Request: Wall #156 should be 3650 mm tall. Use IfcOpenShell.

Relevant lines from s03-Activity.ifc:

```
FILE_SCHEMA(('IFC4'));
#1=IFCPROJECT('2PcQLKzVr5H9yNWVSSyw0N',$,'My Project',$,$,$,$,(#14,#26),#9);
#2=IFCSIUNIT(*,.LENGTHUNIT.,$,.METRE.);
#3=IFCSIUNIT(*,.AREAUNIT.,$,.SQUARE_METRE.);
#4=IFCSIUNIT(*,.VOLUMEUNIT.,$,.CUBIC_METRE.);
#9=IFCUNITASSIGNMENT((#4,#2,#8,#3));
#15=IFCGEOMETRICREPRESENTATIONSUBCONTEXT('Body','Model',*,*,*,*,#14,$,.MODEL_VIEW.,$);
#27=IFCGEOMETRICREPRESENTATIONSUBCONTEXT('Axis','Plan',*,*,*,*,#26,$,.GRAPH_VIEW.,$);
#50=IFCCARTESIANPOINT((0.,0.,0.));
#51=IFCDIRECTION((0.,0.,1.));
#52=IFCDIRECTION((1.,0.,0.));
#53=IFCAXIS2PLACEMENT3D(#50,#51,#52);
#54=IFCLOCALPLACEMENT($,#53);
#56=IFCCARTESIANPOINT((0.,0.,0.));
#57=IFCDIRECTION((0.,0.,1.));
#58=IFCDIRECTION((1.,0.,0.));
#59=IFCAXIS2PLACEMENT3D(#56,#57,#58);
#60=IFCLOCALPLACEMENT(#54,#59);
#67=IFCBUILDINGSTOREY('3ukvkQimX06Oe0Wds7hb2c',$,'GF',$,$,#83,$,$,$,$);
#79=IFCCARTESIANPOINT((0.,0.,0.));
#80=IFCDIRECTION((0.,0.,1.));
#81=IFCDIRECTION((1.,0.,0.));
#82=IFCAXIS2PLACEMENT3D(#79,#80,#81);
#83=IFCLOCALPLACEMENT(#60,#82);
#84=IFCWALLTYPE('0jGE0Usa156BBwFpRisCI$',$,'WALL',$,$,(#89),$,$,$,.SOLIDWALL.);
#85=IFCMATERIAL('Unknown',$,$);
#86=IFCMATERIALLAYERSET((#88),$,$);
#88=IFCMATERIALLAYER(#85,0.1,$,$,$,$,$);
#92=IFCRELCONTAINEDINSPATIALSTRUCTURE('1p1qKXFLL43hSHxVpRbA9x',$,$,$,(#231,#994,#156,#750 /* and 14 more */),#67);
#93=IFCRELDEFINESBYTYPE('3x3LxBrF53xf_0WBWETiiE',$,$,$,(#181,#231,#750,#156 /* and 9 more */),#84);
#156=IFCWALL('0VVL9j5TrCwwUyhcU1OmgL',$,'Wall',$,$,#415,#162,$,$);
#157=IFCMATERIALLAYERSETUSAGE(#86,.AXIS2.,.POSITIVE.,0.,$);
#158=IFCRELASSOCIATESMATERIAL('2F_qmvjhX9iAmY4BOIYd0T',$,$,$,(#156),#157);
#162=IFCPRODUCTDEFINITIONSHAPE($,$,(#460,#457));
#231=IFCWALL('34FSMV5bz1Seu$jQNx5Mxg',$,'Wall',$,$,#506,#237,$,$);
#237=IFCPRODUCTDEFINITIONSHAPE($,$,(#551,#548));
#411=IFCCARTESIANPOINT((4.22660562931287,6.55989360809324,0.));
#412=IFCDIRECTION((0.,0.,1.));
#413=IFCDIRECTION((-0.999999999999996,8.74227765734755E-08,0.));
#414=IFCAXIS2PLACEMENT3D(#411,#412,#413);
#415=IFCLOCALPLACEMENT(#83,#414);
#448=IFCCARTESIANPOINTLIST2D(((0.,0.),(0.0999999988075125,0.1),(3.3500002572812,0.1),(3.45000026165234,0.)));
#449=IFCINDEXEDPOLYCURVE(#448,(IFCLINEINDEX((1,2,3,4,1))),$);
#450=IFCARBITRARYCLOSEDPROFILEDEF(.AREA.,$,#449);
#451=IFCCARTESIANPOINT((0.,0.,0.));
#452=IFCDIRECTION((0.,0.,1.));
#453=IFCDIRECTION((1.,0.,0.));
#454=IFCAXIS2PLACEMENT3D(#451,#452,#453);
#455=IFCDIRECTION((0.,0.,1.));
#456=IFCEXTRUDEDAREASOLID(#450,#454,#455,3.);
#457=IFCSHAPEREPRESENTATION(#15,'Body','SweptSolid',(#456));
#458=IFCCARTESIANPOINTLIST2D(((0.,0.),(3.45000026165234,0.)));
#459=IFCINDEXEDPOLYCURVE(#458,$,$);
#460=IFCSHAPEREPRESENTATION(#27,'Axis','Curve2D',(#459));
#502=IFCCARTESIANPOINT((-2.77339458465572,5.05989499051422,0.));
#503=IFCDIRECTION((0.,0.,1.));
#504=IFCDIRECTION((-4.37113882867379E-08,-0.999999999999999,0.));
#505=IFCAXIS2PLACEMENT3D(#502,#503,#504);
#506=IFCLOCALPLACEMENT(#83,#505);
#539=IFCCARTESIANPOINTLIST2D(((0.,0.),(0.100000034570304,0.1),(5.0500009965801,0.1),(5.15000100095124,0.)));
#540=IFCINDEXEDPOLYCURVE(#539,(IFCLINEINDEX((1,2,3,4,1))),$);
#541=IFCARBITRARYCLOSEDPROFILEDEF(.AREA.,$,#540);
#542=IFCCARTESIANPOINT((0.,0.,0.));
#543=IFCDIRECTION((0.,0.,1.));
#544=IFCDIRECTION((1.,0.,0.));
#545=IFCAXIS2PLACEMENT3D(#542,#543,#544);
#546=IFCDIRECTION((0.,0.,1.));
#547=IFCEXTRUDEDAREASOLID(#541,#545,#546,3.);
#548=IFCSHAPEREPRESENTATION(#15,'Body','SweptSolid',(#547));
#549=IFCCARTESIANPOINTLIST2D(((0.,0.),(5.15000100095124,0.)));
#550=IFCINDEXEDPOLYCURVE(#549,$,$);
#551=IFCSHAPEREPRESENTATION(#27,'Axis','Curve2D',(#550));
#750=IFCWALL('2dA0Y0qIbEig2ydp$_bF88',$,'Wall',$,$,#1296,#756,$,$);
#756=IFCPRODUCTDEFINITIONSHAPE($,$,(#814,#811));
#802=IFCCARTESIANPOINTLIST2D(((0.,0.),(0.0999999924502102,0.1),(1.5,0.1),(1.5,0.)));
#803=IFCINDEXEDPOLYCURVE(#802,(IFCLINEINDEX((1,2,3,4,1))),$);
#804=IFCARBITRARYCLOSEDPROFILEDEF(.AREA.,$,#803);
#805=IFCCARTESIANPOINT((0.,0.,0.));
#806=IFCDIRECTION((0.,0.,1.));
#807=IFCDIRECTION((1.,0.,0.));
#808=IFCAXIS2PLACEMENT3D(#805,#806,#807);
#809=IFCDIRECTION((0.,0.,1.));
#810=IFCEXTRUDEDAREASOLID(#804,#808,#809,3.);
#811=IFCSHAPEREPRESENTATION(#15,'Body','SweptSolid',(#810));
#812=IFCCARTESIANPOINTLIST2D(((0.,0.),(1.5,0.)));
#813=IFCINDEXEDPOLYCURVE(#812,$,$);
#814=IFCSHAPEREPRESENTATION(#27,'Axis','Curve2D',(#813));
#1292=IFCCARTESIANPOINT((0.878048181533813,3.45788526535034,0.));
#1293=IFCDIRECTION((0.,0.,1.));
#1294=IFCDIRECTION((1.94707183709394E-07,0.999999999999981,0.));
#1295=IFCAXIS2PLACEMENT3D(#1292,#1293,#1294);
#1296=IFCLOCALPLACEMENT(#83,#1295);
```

```python
import ifcopenshell
import ifcopenshell.geom
import ifcopenshell.util.representation
import ifcopenshell.util.shape

model = ifcopenshell.open("s03-Activity.ifc")
settings = ifcopenshell.geom.settings()


def volume(element):
    """Net volume in cubic metres, openings subtracted."""
    shape = ifcopenshell.geom.create_shape(settings, element)
    return ifcopenshell.util.shape.get_volume(shape.geometry)


wall = model.by_guid("0VVL9j5TrCwwUyhcU1OmgL")
before = volume(wall)

body = ifcopenshell.util.representation.get_representation(wall, "Model", "Body")
solid = body.Items[0]
old_height = solid.Depth
solid.Depth = 3.65
after = volume(wall)

print(f"height {old_height:g} -> {solid.Depth:g}, volume {before:.3f} -> {after:.3f} m3")

model.write("s03-Activity_edited.ifc")
```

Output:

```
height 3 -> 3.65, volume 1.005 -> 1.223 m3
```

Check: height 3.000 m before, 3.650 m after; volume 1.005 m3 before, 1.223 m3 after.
